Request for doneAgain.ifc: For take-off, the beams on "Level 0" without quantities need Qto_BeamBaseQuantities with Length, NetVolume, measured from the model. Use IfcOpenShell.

First a look at what the model holds.

```python
import ifcopenshell
import ifcopenshell.util.element
import ifcopenshell.util.unit

model = ifcopenshell.open("doneAgain.ifc")
print(model.schema)
for unit_type in ("LENGTHUNIT", "AREAUNIT", "VOLUMEUNIT"):
    print(unit_type, ifcopenshell.util.unit.calculate_unit_scale(model, unit_type))
storey = next(s for s in model.by_type("IfcBuildingStorey") if s.Name == "Level 0")
beams = [e for e in ifcopenshell.util.element.get_decomposition(storey) if e.is_a("IfcBeam")]
for e in sorted(beams, key=lambda e: e.id()):
    print(e.id(), e.is_a(), e.Name, list(ifcopenshell.util.element.get_psets(e, qtos_only=True)), sep=" | ")
```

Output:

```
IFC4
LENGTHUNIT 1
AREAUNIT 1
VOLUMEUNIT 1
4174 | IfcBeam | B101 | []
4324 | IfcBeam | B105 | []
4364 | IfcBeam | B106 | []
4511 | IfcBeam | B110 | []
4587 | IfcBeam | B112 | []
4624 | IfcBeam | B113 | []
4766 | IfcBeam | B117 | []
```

```python
import ifcopenshell
import ifcopenshell.api.pset
import ifcopenshell.geom
import ifcopenshell.util.element
import ifcopenshell.util.shape
import ifcopenshell.util.unit

model = ifcopenshell.open("doneAgain.ifc")
unit_scale = ifcopenshell.util.unit.calculate_unit_scale(model)
volume_scale = ifcopenshell.util.unit.calculate_unit_scale(model, "VOLUMEUNIT")
settings = ifcopenshell.geom.settings()

storey = next(s for s in model.by_type("IfcBuildingStorey") if s.Name == "Level 0")
beams = [e for e in ifcopenshell.util.element.get_decomposition(storey) if e.is_a("IfcBeam")]

for e in sorted(beams, key=lambda e: e.id()):
    if ifcopenshell.util.element.get_psets(e, qtos_only=True, should_inherit=False):
        continue
    # Geometry comes back in metres, in the element's own axes.
    shape = ifcopenshell.geom.create_shape(settings, e)
    values = {
        "Length": ifcopenshell.util.shape.get_max_xyz(shape.geometry) / unit_scale,
        "NetVolume": ifcopenshell.util.shape.get_volume(shape.geometry) / volume_scale,
    }
    qto = ifcopenshell.api.pset.add_qto(model, product=e, name="Qto_BeamBaseQuantities")
    ifcopenshell.api.pset.edit_qto(model, qto=qto, properties=values)
    print(e.id(), {k: round(v, 3) for k, v in values.items()})

model.write("doneAgain_rev.ifc")
```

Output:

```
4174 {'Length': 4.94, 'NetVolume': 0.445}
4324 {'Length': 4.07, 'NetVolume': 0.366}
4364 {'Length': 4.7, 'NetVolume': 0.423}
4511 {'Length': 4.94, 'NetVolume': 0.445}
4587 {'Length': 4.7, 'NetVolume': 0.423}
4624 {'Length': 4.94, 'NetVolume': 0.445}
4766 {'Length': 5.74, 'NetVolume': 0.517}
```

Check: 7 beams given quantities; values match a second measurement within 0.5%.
